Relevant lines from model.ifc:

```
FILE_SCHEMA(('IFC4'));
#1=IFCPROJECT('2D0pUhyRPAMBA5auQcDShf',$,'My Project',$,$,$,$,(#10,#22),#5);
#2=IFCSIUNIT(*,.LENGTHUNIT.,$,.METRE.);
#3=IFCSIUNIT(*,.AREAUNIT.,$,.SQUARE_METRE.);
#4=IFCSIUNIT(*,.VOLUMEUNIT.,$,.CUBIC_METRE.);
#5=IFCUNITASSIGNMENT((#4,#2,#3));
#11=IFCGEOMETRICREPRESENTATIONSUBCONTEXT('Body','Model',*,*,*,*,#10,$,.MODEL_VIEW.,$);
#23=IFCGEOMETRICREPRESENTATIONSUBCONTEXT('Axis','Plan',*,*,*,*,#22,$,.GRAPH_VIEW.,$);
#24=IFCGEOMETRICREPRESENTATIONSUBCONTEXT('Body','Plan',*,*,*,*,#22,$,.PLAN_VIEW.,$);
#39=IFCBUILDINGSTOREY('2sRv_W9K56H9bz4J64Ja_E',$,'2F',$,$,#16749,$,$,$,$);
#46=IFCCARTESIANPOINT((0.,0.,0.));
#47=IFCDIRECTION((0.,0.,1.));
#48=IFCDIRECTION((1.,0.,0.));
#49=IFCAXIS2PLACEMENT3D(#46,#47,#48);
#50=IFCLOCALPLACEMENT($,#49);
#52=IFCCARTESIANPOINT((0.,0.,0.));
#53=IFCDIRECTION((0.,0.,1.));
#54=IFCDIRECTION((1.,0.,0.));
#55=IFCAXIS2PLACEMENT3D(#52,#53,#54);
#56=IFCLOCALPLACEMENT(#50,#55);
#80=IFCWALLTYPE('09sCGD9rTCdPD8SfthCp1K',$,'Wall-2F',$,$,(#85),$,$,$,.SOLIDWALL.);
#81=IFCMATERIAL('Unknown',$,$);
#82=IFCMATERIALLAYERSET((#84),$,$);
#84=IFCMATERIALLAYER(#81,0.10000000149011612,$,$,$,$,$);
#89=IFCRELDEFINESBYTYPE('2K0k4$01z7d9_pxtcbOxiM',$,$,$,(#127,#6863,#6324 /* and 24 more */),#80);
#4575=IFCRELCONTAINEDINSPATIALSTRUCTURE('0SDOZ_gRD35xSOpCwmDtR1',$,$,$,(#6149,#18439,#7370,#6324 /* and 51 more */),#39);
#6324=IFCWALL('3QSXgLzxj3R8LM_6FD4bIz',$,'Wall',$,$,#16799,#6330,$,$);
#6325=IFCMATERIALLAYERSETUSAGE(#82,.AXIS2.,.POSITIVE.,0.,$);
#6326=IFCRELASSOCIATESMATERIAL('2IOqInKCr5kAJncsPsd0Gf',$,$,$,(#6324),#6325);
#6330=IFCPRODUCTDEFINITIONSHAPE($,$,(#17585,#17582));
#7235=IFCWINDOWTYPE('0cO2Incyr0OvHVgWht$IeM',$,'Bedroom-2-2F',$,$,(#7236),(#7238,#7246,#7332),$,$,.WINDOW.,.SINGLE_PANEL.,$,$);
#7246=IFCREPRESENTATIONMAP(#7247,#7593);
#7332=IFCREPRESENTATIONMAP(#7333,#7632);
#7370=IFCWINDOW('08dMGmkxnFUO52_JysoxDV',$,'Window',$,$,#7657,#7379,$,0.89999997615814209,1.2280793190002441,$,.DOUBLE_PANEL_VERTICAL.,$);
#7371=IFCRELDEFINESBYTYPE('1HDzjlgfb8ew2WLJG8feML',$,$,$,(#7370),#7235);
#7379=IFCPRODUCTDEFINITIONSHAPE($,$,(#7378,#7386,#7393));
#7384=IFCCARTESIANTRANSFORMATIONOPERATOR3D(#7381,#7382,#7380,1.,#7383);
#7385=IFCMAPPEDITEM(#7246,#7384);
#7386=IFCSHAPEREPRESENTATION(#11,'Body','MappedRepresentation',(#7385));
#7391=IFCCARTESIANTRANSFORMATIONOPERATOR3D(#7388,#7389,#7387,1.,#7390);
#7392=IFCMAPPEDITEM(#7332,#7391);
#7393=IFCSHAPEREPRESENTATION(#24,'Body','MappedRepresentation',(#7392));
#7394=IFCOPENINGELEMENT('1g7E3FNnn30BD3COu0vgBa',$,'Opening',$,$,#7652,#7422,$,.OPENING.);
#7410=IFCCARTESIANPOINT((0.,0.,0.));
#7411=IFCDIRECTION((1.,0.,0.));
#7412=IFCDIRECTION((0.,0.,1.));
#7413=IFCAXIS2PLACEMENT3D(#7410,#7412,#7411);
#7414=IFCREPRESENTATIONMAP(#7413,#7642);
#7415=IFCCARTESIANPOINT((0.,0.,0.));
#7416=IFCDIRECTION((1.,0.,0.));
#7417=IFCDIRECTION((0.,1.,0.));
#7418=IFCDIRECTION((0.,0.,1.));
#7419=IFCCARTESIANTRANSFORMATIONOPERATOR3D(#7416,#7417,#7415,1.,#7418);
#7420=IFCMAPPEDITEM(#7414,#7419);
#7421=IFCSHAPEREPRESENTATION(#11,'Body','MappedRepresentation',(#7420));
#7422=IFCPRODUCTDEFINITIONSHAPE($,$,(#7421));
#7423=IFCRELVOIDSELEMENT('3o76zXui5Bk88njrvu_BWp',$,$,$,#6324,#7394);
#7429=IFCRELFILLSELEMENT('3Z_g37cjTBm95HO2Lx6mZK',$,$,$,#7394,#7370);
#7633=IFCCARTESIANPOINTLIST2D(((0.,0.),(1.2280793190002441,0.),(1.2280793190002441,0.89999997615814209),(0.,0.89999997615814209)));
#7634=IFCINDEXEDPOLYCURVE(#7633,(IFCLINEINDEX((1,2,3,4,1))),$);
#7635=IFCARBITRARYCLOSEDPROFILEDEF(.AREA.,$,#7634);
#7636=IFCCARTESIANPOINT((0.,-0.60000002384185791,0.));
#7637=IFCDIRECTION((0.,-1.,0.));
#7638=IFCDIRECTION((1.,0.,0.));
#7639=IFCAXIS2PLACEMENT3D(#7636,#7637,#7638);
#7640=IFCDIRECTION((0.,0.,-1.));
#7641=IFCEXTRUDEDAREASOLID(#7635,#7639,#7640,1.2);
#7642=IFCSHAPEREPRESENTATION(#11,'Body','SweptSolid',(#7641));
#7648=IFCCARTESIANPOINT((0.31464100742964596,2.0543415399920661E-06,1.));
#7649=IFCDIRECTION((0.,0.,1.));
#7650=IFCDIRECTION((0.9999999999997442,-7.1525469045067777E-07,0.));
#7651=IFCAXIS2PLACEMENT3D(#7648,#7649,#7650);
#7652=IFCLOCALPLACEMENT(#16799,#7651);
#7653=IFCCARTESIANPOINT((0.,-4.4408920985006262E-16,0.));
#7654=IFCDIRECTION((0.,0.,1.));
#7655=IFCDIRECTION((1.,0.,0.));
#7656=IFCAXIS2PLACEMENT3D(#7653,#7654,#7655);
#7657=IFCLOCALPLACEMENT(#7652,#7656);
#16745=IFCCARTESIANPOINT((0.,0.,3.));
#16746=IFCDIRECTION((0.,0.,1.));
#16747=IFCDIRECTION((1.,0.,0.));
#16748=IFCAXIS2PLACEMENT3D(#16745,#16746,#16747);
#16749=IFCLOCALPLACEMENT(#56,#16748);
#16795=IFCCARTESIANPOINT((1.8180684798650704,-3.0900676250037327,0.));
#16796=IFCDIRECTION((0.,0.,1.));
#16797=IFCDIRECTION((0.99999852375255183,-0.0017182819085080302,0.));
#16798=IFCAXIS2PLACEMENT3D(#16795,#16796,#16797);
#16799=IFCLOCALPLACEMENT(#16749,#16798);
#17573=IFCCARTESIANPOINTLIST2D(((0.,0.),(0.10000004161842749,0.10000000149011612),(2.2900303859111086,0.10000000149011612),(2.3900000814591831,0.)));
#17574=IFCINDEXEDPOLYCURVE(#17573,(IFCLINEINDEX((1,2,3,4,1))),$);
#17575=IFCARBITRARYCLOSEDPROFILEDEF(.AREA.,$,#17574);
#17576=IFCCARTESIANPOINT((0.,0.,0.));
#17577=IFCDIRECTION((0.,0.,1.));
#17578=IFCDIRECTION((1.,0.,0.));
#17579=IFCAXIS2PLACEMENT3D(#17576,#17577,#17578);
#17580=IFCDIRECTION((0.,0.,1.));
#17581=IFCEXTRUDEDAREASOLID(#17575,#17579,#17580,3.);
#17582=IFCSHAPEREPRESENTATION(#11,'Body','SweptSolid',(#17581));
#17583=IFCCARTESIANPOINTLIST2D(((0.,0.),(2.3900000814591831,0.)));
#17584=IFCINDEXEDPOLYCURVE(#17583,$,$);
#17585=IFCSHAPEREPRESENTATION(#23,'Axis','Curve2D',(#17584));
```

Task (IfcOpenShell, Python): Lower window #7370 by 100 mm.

```python
import numpy as np
import ifcopenshell
import ifcopenshell.api.geometry
import ifcopenshell.util.placement
import ifcopenshell.util.unit

model = ifcopenshell.open("model.ifc")
unit_scale = ifcopenshell.util.unit.calculate_unit_scale(model)

window = model.by_guid("08dMGmkxnFUO52_JysoxDV")
opening = window.FillsVoids[0].RelatingOpeningElement
dz = -0.1 / unit_scale

shift = np.array([0.0, 0.0, dz])
# The window is placed relative to its opening, so it follows when the opening moves.
matrix = ifcopenshell.util.placement.get_local_placement(opening.ObjectPlacement)
matrix[:3, 3] += shift
ifcopenshell.api.geometry.edit_object_placement(
    model, product=opening, matrix=matrix, is_si=False, should_transform_children=True
)

print(f"moved by {dz * unit_scale:+.3f} m")

model.write("model_updated.ifc")
```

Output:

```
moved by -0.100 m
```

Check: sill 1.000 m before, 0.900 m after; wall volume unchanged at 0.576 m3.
